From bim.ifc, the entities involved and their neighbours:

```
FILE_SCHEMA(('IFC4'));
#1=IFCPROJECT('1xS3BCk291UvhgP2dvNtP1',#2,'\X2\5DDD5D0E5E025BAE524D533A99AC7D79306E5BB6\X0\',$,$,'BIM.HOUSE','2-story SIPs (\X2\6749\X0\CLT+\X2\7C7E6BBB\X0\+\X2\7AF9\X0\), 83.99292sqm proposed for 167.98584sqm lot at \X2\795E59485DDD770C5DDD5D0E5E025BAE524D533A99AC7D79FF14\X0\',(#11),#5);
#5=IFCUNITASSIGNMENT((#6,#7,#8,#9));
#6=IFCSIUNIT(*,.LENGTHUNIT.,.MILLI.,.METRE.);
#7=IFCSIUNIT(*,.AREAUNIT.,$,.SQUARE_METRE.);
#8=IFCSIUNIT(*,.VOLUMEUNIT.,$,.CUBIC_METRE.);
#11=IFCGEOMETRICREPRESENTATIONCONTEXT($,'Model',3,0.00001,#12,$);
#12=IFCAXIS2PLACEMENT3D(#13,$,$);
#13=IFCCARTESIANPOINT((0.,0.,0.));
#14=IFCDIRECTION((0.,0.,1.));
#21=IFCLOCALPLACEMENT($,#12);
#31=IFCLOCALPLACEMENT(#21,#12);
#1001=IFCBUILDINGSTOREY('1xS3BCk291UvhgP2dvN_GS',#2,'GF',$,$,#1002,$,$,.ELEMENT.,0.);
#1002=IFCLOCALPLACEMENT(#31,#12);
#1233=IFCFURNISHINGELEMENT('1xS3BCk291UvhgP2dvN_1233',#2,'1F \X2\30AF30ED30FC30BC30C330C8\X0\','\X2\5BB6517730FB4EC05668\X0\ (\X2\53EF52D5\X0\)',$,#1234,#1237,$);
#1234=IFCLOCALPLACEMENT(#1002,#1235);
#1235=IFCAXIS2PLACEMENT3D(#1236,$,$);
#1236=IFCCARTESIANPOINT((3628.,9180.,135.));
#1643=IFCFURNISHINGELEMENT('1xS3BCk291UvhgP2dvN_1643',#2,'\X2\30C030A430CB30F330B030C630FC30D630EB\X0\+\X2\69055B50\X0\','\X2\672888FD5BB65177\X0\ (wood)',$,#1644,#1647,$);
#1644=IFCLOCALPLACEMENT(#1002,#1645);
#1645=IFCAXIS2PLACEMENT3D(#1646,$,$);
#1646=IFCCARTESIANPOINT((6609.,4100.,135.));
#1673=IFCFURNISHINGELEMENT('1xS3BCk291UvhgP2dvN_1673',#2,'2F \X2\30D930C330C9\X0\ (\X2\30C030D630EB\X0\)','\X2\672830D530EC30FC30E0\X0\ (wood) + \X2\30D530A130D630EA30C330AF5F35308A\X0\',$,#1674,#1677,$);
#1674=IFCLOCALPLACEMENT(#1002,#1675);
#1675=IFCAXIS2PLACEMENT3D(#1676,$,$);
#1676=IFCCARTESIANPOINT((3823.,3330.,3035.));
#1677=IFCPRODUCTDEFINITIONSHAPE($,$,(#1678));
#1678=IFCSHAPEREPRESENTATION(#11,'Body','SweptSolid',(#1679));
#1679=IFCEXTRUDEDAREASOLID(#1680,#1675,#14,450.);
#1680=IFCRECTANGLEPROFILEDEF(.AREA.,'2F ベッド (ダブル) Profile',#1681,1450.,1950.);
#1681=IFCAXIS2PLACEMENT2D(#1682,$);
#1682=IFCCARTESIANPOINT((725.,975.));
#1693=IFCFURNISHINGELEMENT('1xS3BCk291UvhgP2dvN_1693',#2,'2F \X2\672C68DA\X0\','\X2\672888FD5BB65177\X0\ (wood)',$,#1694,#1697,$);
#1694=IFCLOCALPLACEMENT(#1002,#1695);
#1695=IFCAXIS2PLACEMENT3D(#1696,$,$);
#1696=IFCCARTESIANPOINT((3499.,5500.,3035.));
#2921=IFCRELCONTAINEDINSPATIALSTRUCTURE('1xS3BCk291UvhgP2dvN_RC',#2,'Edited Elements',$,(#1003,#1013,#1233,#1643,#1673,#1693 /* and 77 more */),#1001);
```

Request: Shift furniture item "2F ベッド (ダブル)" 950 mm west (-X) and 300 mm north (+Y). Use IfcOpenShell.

```python
import ifcopenshell
import ifcopenshell.api.geometry
import ifcopenshell.util.placement
import ifcopenshell.util.unit

model = ifcopenshell.open("bim.ifc")
unit_scale = ifcopenshell.util.unit.calculate_unit_scale(model)

item = model.by_guid("1xS3BCk291UvhgP2dvN_1673")
matrix = ifcopenshell.util.placement.get_local_placement(item.ObjectPlacement)
matrix[0, 3] -= 0.95 / unit_scale
matrix[1, 3] += 0.3 / unit_scale
ifcopenshell.api.geometry.edit_object_placement(model, product=item, matrix=matrix, is_si=False)

print(ifcopenshell.util.placement.get_local_placement(item.ObjectPlacement).round(3) + 0.0)

model.write("bim_v2.ifc")
```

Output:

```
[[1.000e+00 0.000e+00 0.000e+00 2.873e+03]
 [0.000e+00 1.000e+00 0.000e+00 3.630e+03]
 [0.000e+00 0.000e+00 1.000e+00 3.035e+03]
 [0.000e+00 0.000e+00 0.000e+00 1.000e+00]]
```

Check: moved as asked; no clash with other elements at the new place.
